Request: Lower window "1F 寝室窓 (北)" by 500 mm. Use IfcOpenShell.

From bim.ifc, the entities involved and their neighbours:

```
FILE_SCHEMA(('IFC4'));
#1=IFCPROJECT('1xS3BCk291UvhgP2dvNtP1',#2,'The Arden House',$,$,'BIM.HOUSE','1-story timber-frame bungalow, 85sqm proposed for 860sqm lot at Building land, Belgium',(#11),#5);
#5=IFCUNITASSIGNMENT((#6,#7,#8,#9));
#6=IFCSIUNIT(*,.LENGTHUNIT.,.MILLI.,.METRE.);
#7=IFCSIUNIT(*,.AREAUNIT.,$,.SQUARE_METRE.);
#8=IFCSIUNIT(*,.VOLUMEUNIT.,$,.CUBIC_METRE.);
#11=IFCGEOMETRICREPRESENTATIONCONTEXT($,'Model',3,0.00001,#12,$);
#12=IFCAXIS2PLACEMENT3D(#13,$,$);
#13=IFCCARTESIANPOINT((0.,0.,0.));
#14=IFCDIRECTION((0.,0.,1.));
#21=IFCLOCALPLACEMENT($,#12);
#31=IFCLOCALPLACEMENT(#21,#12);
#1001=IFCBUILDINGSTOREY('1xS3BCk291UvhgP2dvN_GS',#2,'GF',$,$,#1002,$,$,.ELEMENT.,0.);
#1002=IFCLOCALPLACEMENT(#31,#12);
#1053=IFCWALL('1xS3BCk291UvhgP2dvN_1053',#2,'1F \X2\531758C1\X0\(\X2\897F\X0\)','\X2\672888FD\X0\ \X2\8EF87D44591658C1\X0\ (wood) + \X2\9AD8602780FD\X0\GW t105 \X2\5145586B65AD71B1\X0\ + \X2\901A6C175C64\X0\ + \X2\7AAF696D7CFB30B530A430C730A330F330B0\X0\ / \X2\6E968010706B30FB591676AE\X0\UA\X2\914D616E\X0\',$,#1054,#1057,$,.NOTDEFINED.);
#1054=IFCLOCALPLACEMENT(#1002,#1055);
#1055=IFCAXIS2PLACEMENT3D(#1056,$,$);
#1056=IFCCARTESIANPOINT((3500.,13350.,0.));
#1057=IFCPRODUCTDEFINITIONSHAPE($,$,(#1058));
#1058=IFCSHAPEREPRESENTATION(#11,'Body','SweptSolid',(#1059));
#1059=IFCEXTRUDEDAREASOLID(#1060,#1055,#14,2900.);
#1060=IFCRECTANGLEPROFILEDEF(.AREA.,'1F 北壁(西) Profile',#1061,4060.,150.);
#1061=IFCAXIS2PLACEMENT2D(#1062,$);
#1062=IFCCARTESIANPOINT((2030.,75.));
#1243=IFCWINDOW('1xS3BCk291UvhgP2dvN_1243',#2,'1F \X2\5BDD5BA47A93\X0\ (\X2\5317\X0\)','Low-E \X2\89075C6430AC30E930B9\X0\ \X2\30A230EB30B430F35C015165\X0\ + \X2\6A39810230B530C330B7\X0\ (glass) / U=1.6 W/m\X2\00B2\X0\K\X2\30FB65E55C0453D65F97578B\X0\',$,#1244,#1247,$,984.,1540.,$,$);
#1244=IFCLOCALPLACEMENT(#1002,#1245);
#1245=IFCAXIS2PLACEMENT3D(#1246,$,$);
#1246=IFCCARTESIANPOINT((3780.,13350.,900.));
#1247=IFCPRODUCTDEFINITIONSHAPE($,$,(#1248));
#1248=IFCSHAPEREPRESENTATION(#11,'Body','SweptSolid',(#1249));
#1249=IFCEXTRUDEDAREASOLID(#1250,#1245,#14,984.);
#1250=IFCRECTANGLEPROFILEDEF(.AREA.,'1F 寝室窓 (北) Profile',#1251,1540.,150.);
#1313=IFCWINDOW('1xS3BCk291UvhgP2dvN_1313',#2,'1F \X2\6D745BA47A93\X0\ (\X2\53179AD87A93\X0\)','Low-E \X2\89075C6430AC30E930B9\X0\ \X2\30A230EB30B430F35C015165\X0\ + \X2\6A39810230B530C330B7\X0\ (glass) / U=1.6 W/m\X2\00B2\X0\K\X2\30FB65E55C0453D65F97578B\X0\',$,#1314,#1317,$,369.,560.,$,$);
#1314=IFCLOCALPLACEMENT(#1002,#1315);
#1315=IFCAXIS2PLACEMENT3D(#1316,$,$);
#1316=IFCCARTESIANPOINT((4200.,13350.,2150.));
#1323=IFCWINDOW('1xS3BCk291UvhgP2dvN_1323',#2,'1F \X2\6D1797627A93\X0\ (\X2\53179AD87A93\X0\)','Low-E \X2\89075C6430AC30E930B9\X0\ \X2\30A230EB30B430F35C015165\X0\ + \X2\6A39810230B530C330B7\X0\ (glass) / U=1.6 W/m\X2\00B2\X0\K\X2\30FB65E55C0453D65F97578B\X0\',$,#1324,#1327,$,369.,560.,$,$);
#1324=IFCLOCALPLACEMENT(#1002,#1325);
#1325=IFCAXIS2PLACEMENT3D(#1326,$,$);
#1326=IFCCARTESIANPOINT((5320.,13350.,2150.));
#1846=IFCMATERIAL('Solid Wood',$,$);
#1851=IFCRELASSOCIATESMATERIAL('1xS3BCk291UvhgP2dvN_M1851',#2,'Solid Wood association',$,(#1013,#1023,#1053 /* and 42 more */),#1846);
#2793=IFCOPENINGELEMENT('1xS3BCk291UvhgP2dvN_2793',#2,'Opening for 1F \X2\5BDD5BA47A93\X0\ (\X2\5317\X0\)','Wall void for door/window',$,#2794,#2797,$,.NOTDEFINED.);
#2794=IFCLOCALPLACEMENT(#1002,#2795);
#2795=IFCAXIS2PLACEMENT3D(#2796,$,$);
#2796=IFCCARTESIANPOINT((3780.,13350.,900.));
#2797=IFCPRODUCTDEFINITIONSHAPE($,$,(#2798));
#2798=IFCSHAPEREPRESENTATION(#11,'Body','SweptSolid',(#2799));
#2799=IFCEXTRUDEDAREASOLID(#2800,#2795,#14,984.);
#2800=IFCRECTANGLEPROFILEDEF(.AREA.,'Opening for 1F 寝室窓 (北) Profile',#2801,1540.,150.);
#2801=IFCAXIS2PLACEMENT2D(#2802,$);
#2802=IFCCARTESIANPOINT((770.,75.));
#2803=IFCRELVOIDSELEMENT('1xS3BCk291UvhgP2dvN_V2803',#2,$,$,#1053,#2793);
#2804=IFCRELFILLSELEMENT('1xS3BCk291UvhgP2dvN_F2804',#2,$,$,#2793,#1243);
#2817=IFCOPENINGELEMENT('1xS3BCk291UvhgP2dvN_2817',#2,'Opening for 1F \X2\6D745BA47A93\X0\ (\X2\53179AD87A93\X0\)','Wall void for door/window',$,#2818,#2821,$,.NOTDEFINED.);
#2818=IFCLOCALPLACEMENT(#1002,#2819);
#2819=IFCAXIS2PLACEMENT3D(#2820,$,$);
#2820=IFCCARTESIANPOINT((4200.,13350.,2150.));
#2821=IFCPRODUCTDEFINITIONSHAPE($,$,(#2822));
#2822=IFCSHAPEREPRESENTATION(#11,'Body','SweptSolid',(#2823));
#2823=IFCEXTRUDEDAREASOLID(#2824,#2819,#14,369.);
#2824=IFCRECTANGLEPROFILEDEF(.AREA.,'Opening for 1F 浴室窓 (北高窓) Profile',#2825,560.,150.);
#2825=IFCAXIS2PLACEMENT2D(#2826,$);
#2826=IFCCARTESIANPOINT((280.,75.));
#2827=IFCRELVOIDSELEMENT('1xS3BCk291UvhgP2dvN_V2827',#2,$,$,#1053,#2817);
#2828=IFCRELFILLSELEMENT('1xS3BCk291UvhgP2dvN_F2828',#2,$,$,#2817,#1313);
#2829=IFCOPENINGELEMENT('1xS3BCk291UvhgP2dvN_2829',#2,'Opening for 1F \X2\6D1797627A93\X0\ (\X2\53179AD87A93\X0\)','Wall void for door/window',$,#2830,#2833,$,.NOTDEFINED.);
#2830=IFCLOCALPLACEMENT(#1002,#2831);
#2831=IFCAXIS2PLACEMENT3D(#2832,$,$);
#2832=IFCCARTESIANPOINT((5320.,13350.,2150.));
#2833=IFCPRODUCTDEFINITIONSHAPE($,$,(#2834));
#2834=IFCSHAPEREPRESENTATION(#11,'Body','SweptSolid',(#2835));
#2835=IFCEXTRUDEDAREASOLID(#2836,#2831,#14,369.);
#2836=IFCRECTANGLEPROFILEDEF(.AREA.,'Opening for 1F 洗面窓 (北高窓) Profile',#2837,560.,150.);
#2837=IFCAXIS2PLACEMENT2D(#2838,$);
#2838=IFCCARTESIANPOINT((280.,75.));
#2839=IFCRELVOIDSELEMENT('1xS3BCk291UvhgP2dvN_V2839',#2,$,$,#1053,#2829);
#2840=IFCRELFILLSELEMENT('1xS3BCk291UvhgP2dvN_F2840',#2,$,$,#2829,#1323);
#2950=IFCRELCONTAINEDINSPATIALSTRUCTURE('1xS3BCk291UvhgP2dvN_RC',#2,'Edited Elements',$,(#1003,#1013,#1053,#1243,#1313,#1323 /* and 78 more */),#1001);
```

```python
import numpy as np
import ifcopenshell
import ifcopenshell.api.geometry
import ifcopenshell.util.placement
import ifcopenshell.util.unit

model = ifcopenshell.open("bim.ifc")
unit_scale = ifcopenshell.util.unit.calculate_unit_scale(model)

window = model.by_guid("1xS3BCk291UvhgP2dvN_1243")
opening = window.FillsVoids[0].RelatingOpeningElement
dz = -500.0

shift = np.array([0.0, 0.0, dz])
# The window is not placed relative to its opening, so move both.
for product in (opening, window):
    matrix = ifcopenshell.util.placement.get_local_placement(product.ObjectPlacement)
    matrix[:3, 3] += shift
    ifcopenshell.api.geometry.edit_object_placement(model, product=product, matrix=matrix, is_si=False)

print(f"moved by {dz * unit_scale:+.3f} m")

model.write("bim_rev.ifc")
```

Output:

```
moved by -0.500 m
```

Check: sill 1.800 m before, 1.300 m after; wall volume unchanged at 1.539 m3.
